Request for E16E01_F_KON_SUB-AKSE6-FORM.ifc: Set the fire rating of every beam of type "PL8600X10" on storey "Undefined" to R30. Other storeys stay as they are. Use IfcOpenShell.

First a look at what the model holds.

```python
import ifcopenshell
import ifcopenshell.util.element

model = ifcopenshell.open("E16E01_F_KON_SUB-AKSE6-FORM.ifc")
print(model.schema)
storey = next(s for s in model.by_type("IfcBuildingStorey") if s.Name == "Undefined")
beams = [e for e in ifcopenshell.util.element.get_decomposition(storey) if e.is_a("IfcBeam")]
seen = {}
for e in beams:
    element_type = ifcopenshell.util.element.get_type(e)
    key = (element_type.Name if element_type != e and element_type else None, ifcopenshell.util.element.get_pset(e, "Pset_BeamCommon", "FireRating"))
    seen[key] = seen.get(key, 0) + 1
for (name, value), count in sorted(seen.items(), key=str):
    print(count, "x", name, "|", value)
```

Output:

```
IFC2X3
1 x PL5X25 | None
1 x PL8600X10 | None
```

```python
import ifcopenshell
import ifcopenshell.api.pset
import ifcopenshell.util.element

model = ifcopenshell.open("E16E01_F_KON_SUB-AKSE6-FORM.ifc")

storey = next(s for s in model.by_type("IfcBuildingStorey") if s.Name == "Undefined")
beams = [e for e in ifcopenshell.util.element.get_decomposition(storey) if e.is_a("IfcBeam")]

count = 0
for e in beams:
    element_type = ifcopenshell.util.element.get_type(e)
    if element_type in (None, e) or element_type.Name != "PL8600X10":
        continue
    # add_pset returns the element's existing set when there is one.
    pset = ifcopenshell.api.pset.add_pset(model, product=e, name="Pset_BeamCommon")
    ifcopenshell.api.pset.edit_pset(model, pset=pset, properties={"FireRating": "R30"})
    count += 1

print(count, "beams updated")

model.write("E16E01_F_KON_SUB-AKSE6-FORM_updated.ifc")
```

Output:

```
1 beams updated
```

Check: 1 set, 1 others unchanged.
